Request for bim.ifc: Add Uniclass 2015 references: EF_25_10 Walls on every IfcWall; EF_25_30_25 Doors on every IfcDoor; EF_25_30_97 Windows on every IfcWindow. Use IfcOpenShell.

First a look at what the model holds.

```python
import ifcopenshell

model = ifcopenshell.open("bim.ifc")
print(model.schema)
print("classifications:", [c.Name for c in model.by_type("IfcClassification")])
for ifc_class in ("IfcDoor", "IfcRoof", "IfcStair", "IfcWall", "IfcWindow"):
    print(ifc_class, len(model.by_type(ifc_class)))
```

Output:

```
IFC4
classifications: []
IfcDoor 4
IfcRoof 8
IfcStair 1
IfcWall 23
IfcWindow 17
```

```python
import ifcopenshell
import ifcopenshell.api.classification

model = ifcopenshell.open("bim.ifc")

system = ifcopenshell.api.classification.add_classification(model, classification="Uniclass 2015")

codes = {
    "IfcWall": ("EF_25_10", "Walls"),
    "IfcDoor": ("EF_25_30_25", "Doors"),
    "IfcWindow": ("EF_25_30_97", "Windows"),
}
for ifc_class, (code, name) in codes.items():
    products = model.by_type(ifc_class)
    ifcopenshell.api.classification.add_reference(
        model, products=products, classification=system, identification=code, name=name
    )
    print(code, len(products))

model.write("bim_rev.ifc")
```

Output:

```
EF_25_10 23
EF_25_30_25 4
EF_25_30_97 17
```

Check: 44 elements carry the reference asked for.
